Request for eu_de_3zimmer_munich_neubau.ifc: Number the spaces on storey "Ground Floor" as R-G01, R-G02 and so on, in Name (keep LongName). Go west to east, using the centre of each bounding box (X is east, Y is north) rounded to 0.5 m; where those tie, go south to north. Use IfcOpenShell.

First a look at what the model holds.

```python
import ifcopenshell
import ifcopenshell.util.element
import ifcopenshell.util.placement

model = ifcopenshell.open("eu_de_3zimmer_munich_neubau.ifc")
print(model.schema)
storey = next(s for s in model.by_type("IfcBuildingStorey") if s.Name == "Ground Floor")
spaces = [e for e in ifcopenshell.util.element.get_decomposition(storey) if e.is_a("IfcSpace")]
for e in sorted(spaces, key=lambda e: e.id()):
    origin = ifcopenshell.util.placement.get_local_placement(e.ObjectPlacement)[:3, 3]
    print(e.id(), e.Name, e.LongName, origin.round(2) + 0.0, sep=" | ")
```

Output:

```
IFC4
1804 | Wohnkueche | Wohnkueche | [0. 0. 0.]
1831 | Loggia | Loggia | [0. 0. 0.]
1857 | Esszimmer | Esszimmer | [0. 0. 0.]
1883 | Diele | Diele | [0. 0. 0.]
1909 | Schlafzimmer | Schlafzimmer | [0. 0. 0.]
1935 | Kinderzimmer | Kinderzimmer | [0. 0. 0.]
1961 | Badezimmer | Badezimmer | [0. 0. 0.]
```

```python
import ifcopenshell
import ifcopenshell.geom
import ifcopenshell.util.element
import ifcopenshell.util.shape

model = ifcopenshell.open("eu_de_3zimmer_munich_neubau.ifc")
settings = ifcopenshell.geom.settings()
settings.set("use-world-coords", True)


def centre(element):
    shape = ifcopenshell.geom.create_shape(settings, element)
    return ifcopenshell.util.shape.get_bbox_centroid(shape.geometry)


storey = next(s for s in model.by_type("IfcBuildingStorey") if s.Name == "Ground Floor")
spaces = [e for e in ifcopenshell.util.element.get_decomposition(storey) if e.is_a("IfcSpace")]

# Insertion points can sit at a corner or the storey origin, so sort by the geometry (in metres).
centres = {e: centre(e) for e in spaces}
spaces.sort(key=lambda e: (round(centres[e][0] / 0.5), centres[e][1]))

for i, e in enumerate(spaces, start=1):
    number = f"R-G{i:02d}"
    e.Name = number
    print(e.id(), number)

model.write("eu_de_3zimmer_munich_neubau_edited.ifc")
```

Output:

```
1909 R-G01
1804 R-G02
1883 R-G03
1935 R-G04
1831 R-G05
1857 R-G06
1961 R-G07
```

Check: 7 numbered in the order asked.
